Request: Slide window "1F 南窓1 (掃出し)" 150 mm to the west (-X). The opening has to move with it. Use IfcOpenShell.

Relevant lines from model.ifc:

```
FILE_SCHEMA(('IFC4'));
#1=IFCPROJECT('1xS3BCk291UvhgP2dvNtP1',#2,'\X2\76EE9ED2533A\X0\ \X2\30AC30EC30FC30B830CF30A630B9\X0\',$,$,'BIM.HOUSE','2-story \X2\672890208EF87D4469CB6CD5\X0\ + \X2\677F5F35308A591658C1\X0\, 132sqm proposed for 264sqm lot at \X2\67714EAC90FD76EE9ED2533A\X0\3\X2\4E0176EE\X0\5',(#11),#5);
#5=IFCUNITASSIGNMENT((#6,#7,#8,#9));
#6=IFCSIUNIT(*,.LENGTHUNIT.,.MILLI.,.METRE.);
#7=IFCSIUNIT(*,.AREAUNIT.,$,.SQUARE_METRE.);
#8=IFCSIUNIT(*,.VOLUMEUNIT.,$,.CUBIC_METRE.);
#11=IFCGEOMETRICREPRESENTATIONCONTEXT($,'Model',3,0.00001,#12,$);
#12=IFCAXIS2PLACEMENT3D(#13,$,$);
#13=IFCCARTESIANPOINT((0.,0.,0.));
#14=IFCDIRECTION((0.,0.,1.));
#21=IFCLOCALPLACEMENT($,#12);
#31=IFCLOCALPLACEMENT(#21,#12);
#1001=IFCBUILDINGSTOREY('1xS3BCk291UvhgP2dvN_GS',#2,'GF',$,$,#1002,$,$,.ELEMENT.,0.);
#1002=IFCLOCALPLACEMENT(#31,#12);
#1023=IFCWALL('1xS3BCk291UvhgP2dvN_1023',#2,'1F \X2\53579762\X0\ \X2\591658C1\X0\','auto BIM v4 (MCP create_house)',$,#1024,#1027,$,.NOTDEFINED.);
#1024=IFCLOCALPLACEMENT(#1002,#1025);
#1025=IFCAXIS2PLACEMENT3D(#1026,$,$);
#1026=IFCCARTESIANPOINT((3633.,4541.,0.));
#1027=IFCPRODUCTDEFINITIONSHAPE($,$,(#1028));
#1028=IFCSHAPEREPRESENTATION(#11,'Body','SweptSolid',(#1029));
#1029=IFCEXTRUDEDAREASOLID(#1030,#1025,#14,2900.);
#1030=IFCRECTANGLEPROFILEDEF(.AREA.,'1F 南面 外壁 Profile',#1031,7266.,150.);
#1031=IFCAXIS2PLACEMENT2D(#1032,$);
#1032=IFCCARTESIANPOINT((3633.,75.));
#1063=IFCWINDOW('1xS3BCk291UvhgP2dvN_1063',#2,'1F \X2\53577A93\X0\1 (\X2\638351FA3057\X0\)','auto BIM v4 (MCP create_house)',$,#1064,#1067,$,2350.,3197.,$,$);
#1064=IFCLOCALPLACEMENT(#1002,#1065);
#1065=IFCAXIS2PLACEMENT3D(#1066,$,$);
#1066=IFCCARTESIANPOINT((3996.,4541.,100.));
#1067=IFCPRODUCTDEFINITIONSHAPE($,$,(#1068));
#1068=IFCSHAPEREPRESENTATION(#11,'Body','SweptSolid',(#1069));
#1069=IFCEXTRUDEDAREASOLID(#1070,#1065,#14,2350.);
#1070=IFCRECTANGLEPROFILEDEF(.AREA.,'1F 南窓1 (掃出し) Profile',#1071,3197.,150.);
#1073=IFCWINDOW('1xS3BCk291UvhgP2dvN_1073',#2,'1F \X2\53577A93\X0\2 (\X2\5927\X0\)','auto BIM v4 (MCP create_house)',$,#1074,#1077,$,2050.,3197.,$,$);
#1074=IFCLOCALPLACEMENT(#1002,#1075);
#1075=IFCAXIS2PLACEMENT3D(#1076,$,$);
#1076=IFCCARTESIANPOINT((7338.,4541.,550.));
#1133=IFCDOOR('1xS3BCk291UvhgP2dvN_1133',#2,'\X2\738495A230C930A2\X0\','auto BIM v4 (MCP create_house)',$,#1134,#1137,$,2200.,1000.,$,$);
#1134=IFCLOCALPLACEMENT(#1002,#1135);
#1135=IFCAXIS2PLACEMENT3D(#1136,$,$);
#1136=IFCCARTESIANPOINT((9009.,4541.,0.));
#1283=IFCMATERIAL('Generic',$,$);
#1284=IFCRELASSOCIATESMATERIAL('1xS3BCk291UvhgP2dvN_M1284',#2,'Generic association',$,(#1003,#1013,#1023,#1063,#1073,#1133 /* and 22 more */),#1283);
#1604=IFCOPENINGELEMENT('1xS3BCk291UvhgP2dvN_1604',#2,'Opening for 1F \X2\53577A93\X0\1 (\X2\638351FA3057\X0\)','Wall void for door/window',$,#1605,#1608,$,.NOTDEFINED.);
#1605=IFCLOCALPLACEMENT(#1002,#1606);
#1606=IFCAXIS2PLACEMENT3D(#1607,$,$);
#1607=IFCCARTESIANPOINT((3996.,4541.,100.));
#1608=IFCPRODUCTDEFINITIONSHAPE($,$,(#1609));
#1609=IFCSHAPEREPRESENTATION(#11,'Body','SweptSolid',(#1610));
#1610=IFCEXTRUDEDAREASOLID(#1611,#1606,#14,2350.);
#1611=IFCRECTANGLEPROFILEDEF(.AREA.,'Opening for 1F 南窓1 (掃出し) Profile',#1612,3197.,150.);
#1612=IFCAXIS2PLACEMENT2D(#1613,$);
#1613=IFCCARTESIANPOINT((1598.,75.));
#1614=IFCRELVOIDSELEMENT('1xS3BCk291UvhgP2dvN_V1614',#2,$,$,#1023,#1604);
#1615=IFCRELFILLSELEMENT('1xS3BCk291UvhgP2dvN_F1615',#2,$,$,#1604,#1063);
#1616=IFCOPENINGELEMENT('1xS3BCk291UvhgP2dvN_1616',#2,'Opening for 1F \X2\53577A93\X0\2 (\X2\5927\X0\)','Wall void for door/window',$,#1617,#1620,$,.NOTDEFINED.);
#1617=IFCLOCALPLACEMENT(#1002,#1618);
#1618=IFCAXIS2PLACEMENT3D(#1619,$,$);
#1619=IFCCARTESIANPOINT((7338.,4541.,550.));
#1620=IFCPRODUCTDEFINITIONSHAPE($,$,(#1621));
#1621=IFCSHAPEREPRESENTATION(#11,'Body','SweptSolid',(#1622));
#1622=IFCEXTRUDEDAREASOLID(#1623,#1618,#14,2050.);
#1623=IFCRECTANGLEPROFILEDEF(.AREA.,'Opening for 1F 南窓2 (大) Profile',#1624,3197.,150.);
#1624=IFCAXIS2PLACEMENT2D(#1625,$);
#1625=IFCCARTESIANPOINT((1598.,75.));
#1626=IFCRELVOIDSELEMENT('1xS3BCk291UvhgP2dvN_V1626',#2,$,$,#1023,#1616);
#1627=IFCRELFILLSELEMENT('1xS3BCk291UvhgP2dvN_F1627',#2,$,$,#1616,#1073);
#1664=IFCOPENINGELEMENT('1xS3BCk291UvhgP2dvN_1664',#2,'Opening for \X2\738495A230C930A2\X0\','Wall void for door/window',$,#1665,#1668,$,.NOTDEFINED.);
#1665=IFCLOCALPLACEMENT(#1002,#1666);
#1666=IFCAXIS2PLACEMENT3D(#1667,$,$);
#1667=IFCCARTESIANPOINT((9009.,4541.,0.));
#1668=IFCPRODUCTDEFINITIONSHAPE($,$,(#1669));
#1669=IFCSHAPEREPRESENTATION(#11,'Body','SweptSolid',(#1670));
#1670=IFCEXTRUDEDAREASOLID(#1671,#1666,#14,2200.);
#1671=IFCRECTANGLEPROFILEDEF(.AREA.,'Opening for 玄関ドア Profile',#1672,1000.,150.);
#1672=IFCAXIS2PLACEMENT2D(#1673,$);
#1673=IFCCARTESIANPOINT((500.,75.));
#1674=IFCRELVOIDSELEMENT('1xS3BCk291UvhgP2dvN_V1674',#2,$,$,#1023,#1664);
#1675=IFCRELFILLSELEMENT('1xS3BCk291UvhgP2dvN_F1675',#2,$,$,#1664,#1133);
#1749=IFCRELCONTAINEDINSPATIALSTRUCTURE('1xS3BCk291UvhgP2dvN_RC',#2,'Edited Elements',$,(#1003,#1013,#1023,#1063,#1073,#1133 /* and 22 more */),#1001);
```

```python
import ifcopenshell
import ifcopenshell.api.geometry
import ifcopenshell.util.placement
import ifcopenshell.util.unit

model = ifcopenshell.open("model.ifc")
unit_scale = ifcopenshell.util.unit.calculate_unit_scale(model)

window = model.by_guid("1xS3BCk291UvhgP2dvN_1063")
opening = window.FillsVoids[0].RelatingOpeningElement
wall = opening.VoidsElements[0].RelatingBuildingElement

wall_matrix = ifcopenshell.util.placement.get_local_placement(wall.ObjectPlacement)
shift = wall_matrix[:3, 0] * -0.15 / unit_scale
before = ifcopenshell.util.placement.get_local_placement(window.ObjectPlacement)[:3, 3].copy()

# The window is not placed relative to its opening, so move both.
for product in (opening, window):
    matrix = ifcopenshell.util.placement.get_local_placement(product.ObjectPlacement)
    matrix[:3, 3] += shift
    ifcopenshell.api.geometry.edit_object_placement(model, product=product, matrix=matrix, is_si=False)

after = ifcopenshell.util.placement.get_local_placement(window.ObjectPlacement)[:3, 3]
print("window moved by", (after - before).round(3) + 0.0)

model.write("model_v2.ifc")
```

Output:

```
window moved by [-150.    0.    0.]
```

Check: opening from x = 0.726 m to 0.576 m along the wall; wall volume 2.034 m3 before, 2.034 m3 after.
